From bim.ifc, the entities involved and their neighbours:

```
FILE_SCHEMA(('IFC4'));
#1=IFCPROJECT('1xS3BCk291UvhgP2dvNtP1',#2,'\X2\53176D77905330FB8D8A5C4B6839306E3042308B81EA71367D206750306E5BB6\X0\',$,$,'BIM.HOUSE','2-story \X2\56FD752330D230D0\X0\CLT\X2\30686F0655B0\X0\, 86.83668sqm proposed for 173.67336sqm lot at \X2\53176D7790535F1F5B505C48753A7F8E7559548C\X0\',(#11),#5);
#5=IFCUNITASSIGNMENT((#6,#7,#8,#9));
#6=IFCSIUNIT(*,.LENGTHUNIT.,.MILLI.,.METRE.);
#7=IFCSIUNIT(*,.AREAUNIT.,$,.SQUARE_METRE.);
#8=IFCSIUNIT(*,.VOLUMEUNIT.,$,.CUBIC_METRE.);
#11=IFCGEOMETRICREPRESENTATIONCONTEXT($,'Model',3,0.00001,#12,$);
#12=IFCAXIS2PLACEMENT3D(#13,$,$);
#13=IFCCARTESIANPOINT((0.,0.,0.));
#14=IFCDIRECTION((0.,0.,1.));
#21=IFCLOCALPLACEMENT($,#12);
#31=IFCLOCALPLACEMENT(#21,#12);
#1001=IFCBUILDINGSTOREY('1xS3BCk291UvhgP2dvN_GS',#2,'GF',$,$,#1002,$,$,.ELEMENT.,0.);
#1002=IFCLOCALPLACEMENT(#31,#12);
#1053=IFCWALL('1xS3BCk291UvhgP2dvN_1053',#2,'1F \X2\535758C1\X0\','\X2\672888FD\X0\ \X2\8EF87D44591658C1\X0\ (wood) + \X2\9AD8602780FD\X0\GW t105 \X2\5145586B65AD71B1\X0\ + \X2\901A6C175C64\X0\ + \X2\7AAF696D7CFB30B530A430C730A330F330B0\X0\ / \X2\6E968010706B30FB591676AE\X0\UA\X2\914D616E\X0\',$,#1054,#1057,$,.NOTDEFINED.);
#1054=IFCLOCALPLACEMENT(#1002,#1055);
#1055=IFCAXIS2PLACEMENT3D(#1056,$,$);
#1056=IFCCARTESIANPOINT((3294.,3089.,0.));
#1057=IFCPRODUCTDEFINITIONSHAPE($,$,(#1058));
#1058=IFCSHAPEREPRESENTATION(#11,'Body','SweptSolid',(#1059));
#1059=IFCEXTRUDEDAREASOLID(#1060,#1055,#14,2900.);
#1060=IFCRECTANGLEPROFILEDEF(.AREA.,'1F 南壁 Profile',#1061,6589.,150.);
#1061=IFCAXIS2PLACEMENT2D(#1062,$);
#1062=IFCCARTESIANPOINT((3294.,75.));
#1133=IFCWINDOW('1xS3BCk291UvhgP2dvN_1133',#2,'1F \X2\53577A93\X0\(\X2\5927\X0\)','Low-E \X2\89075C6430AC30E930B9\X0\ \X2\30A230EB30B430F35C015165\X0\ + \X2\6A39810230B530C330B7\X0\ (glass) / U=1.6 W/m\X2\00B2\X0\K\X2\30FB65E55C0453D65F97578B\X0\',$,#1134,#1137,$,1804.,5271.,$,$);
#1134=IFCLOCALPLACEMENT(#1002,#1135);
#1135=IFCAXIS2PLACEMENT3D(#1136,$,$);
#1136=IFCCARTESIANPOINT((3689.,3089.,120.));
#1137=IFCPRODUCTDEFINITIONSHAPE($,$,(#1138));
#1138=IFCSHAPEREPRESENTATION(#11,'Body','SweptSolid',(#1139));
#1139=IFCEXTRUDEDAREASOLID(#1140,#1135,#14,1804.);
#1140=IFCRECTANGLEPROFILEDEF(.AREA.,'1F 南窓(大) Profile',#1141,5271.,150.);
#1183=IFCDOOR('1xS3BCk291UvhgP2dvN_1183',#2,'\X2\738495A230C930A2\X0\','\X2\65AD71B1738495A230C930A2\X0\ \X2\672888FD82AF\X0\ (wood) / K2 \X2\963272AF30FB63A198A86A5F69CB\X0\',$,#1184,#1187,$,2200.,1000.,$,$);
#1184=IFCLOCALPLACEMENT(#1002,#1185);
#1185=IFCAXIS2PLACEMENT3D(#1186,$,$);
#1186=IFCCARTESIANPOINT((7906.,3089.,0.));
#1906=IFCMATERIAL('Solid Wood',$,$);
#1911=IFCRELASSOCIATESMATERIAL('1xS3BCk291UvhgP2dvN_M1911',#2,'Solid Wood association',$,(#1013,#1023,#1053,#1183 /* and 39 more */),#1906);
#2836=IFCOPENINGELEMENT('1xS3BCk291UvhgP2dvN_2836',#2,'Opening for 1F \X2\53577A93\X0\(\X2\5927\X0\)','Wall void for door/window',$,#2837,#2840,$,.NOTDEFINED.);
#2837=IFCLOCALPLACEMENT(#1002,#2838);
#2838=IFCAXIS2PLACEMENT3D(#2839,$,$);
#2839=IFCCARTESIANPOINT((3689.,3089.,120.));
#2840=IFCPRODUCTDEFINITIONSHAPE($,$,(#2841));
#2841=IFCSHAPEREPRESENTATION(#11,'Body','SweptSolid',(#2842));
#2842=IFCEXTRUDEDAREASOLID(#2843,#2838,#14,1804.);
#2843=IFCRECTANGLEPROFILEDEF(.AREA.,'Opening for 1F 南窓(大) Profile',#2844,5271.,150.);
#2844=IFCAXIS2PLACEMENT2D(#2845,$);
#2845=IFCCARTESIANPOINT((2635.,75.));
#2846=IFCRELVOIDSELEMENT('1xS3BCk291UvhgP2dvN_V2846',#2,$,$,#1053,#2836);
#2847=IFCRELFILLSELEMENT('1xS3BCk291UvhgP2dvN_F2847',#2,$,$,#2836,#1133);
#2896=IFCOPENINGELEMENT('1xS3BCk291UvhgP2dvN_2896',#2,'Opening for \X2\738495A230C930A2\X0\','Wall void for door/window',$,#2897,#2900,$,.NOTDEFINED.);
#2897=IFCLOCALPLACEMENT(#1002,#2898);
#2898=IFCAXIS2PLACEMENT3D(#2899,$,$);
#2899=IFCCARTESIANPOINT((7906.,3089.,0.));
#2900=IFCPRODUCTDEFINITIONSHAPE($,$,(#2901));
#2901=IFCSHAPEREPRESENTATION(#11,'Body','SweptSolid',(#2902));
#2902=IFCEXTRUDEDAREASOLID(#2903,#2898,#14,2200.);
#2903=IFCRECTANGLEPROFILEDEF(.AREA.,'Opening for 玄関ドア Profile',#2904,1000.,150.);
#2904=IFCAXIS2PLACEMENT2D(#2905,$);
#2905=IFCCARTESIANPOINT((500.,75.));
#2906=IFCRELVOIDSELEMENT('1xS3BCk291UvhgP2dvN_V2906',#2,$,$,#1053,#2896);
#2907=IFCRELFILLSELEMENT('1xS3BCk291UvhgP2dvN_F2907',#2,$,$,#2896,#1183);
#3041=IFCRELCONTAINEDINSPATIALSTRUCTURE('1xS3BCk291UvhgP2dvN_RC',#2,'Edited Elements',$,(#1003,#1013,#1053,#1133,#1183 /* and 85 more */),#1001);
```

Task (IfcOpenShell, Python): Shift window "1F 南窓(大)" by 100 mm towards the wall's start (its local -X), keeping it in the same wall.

```python
import ifcopenshell
import ifcopenshell.api.geometry
import ifcopenshell.util.placement
import ifcopenshell.util.unit

model = ifcopenshell.open("bim.ifc")
unit_scale = ifcopenshell.util.unit.calculate_unit_scale(model)

window = model.by_id(1133)
opening = window.FillsVoids[0].RelatingOpeningElement
wall = opening.VoidsElements[0].RelatingBuildingElement

wall_matrix = ifcopenshell.util.placement.get_local_placement(wall.ObjectPlacement)
shift = wall_matrix[:3, 0] * -0.1 / unit_scale
before = ifcopenshell.util.placement.get_local_placement(window.ObjectPlacement)[:3, 3].copy()

# The window is not placed relative to its opening, so move both.
for product in (opening, window):
    matrix = ifcopenshell.util.placement.get_local_placement(product.ObjectPlacement)
    matrix[:3, 3] += shift
    ifcopenshell.api.geometry.edit_object_placement(model, product=product, matrix=matrix, is_si=False)

after = ifcopenshell.util.placement.get_local_placement(window.ObjectPlacement)[:3, 3]
print("window moved by", (after - before).round(3) + 0.0)

model.write("bim_rev.ifc")
```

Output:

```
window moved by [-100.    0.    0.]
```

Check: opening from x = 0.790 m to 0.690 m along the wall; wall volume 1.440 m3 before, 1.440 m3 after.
